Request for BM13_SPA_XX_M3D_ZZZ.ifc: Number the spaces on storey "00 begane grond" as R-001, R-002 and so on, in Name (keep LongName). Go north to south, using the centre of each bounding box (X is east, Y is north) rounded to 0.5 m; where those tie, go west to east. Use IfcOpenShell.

First a look at what the model holds.

```python
import ifcopenshell
import ifcopenshell.util.element
import ifcopenshell.util.placement

model = ifcopenshell.open("BM13_SPA_XX_M3D_ZZZ.ifc")
print(model.schema)
storey = next(s for s in model.by_type("IfcBuildingStorey") if s.Name == "00 begane grond")
spaces = [e for e in ifcopenshell.util.element.get_decomposition(storey) if e.is_a("IfcSpace")]
for e in sorted(spaces, key=lambda e: e.id()):
    origin = ifcopenshell.util.placement.get_local_placement(e.ObjectPlacement)[:3, 3]
    print(e.id(), e.Name, e.LongName, origin.round(2) + 0.0, sep=" | ")
```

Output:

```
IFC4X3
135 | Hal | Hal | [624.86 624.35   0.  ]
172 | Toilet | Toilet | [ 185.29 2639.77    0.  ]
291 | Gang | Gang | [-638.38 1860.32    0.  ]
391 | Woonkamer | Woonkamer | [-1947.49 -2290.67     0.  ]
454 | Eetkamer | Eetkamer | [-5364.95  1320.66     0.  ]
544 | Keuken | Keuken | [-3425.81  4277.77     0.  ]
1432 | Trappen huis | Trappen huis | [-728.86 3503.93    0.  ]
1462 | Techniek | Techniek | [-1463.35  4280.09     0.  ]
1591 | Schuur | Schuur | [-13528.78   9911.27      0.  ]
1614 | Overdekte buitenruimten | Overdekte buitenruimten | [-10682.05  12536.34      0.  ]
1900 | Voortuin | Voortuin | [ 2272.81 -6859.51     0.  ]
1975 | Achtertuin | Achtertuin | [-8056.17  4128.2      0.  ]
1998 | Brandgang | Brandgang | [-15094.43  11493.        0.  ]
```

```python
import ifcopenshell
import ifcopenshell.geom
import ifcopenshell.util.element
import ifcopenshell.util.shape

model = ifcopenshell.open("BM13_SPA_XX_M3D_ZZZ.ifc")
settings = ifcopenshell.geom.settings()
settings.set("use-world-coords", True)


def centre(element):
    shape = ifcopenshell.geom.create_shape(settings, element)
    return ifcopenshell.util.shape.get_bbox_centroid(shape.geometry)


storey = next(s for s in model.by_type("IfcBuildingStorey") if s.Name == "00 begane grond")
spaces = [e for e in ifcopenshell.util.element.get_decomposition(storey) if e.is_a("IfcSpace")]

# Insertion points can sit at a corner or the storey origin, so sort by the geometry (in metres).
centres = {e: centre(e) for e in spaces}
spaces.sort(key=lambda e: (-round(centres[e][1] / 0.5), centres[e][0]))

for i, e in enumerate(spaces, start=1):
    number = f"R-0{i:02d}"
    e.Name = number
    print(e.id(), number)

model.write("BM13_SPA_XX_M3D_ZZZ_edited.ifc")
```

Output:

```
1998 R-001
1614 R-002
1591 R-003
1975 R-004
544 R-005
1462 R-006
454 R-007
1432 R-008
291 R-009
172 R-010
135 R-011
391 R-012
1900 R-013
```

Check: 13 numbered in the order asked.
